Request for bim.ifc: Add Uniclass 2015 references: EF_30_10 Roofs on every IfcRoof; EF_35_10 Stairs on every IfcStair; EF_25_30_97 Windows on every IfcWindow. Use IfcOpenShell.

First a look at what the model holds.

```python
import ifcopenshell

model = ifcopenshell.open("bim.ifc")
print(model.schema)
print("classifications:", [c.Name for c in model.by_type("IfcClassification")])
for ifc_class in ("IfcDoor", "IfcRoof", "IfcStair", "IfcWall", "IfcWindow"):
    print(ifc_class, len(model.by_type(ifc_class)))
```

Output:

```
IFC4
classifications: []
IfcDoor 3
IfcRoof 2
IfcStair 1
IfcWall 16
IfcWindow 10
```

```python
import ifcopenshell
import ifcopenshell.api.classification

model = ifcopenshell.open("bim.ifc")

system = ifcopenshell.api.classification.add_classification(model, classification="Uniclass 2015")

codes = {
    "IfcRoof": ("EF_30_10", "Roofs"),
    "IfcStair": ("EF_35_10", "Stairs"),
    "IfcWindow": ("EF_25_30_97", "Windows"),
}
for ifc_class, (code, name) in codes.items():
    products = model.by_type(ifc_class)
    ifcopenshell.api.classification.add_reference(
        model, products=products, classification=system, identification=code, name=name
    )
    print(code, len(products))

model.write("bim_v2.ifc")
```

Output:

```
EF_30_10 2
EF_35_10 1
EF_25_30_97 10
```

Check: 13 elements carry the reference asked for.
